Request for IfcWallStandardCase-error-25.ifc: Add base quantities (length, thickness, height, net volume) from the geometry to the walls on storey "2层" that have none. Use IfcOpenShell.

First a look at what the model holds.

```python
import ifcopenshell
import ifcopenshell.util.element
import ifcopenshell.util.unit

model = ifcopenshell.open("IfcWallStandardCase-error-25.ifc")
print(model.schema)
for unit_type in ("LENGTHUNIT", "AREAUNIT", "VOLUMEUNIT"):
    print(unit_type, ifcopenshell.util.unit.calculate_unit_scale(model, unit_type))
storey = next(s for s in model.by_type("IfcBuildingStorey") if s.Name == "2层")
walls = [e for e in ifcopenshell.util.element.get_decomposition(storey) if e.is_a("IfcWall")]
for e in sorted(walls, key=lambda e: e.id()):
    print(e.id(), e.is_a(), e.Name, list(ifcopenshell.util.element.get_psets(e, qtos_only=True)), sep=" | ")
```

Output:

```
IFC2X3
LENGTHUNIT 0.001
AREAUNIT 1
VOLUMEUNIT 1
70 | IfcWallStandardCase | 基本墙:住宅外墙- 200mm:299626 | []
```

```python
import ifcopenshell
import ifcopenshell.api.pset
import ifcopenshell.geom
import ifcopenshell.util.element
import ifcopenshell.util.shape
import ifcopenshell.util.unit

model = ifcopenshell.open("IfcWallStandardCase-error-25.ifc")
unit_scale = ifcopenshell.util.unit.calculate_unit_scale(model)
volume_scale = ifcopenshell.util.unit.calculate_unit_scale(model, "VOLUMEUNIT")
settings = ifcopenshell.geom.settings()

storey = next(s for s in model.by_type("IfcBuildingStorey") if s.Name == "2层")
walls = [e for e in ifcopenshell.util.element.get_decomposition(storey) if e.is_a("IfcWall")]

for e in sorted(walls, key=lambda e: e.id()):
    if ifcopenshell.util.element.get_psets(e, qtos_only=True, should_inherit=False):
        continue
    # Geometry comes back in metres, in the element's own axes.
    shape = ifcopenshell.geom.create_shape(settings, e)
    values = {
        "Length": ifcopenshell.util.shape.get_x(shape.geometry) / unit_scale,
        "Width": ifcopenshell.util.shape.get_y(shape.geometry) / unit_scale,
        "Height": ifcopenshell.util.shape.get_z(shape.geometry) / unit_scale,
        "NetVolume": ifcopenshell.util.shape.get_volume(shape.geometry) / volume_scale,
    }
    qto = ifcopenshell.api.pset.add_qto(model, product=e, name="BaseQuantities")
    ifcopenshell.api.pset.edit_qto(model, qto=qto, properties=values)
    print(e.id(), {k: round(v, 3) for k, v in values.items()})

model.write("IfcWallStandardCase-error-25_v2.ifc")
```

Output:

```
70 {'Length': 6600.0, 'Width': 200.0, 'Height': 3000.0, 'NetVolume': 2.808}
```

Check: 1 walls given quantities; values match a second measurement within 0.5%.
